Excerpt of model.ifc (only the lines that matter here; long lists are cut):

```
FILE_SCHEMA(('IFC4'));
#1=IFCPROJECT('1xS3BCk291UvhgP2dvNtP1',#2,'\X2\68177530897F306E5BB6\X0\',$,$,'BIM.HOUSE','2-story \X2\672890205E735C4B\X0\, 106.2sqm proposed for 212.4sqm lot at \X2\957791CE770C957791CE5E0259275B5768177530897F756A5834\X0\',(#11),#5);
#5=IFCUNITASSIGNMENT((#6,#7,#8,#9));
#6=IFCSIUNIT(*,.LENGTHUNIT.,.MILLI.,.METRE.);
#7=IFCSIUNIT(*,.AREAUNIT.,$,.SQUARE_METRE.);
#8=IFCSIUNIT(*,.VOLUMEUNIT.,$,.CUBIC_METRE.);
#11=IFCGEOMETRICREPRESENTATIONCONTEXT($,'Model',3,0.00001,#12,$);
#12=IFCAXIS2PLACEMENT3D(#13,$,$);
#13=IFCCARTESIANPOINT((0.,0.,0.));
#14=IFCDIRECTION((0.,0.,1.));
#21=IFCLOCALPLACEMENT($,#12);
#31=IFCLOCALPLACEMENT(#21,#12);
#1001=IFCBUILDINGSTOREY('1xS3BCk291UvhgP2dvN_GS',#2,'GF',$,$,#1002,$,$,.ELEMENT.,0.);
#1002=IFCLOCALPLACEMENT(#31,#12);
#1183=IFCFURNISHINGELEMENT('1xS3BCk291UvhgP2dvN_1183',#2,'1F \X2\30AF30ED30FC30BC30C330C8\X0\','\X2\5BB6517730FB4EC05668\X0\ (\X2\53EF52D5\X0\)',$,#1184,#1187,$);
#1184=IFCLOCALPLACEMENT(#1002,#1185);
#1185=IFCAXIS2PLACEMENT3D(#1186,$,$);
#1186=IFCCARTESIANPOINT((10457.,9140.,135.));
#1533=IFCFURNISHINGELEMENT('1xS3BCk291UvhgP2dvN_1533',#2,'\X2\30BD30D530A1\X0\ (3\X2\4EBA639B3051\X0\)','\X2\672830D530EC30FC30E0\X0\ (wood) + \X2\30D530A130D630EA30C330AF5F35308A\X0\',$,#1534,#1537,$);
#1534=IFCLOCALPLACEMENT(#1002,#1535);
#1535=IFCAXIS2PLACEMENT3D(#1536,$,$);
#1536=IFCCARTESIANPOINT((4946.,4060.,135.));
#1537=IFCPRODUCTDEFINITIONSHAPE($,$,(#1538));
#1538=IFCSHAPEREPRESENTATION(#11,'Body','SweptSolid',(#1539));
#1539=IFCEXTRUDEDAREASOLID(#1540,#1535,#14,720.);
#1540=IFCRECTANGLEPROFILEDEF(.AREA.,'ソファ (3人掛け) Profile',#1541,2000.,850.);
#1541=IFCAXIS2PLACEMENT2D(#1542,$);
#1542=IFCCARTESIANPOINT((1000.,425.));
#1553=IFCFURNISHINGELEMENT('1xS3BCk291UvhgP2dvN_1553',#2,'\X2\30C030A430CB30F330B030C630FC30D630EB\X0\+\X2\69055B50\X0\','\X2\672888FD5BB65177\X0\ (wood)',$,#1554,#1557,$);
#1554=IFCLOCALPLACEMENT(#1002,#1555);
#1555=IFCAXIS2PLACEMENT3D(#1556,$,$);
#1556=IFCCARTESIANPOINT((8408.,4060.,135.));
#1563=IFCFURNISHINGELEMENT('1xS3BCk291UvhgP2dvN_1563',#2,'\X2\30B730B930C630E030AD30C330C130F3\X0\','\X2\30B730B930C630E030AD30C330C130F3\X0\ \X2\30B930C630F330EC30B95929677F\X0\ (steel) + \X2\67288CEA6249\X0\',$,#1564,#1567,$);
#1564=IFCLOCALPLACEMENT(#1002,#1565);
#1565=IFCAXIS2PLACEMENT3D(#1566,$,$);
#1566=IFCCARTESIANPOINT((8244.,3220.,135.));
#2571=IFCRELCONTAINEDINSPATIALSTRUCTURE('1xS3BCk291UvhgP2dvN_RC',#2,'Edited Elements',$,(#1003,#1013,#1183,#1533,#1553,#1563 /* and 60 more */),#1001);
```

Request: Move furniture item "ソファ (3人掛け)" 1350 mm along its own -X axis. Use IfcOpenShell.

```python
import ifcopenshell
import ifcopenshell.api.geometry
import ifcopenshell.util.placement
import ifcopenshell.util.unit

model = ifcopenshell.open("model.ifc")
unit_scale = ifcopenshell.util.unit.calculate_unit_scale(model)

item = model.by_id(1533)
matrix = ifcopenshell.util.placement.get_local_placement(item.ObjectPlacement)
matrix[:3, 3] -= matrix[:3, 0] * 1.35 / unit_scale
ifcopenshell.api.geometry.edit_object_placement(model, product=item, matrix=matrix, is_si=False)

print(ifcopenshell.util.placement.get_local_placement(item.ObjectPlacement).round(3) + 0.0)

model.write("model_v2.ifc")
```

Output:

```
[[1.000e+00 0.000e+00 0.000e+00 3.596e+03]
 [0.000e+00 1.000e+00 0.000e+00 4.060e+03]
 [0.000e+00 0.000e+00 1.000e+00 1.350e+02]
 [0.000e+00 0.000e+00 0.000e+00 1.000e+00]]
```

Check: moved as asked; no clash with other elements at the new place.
